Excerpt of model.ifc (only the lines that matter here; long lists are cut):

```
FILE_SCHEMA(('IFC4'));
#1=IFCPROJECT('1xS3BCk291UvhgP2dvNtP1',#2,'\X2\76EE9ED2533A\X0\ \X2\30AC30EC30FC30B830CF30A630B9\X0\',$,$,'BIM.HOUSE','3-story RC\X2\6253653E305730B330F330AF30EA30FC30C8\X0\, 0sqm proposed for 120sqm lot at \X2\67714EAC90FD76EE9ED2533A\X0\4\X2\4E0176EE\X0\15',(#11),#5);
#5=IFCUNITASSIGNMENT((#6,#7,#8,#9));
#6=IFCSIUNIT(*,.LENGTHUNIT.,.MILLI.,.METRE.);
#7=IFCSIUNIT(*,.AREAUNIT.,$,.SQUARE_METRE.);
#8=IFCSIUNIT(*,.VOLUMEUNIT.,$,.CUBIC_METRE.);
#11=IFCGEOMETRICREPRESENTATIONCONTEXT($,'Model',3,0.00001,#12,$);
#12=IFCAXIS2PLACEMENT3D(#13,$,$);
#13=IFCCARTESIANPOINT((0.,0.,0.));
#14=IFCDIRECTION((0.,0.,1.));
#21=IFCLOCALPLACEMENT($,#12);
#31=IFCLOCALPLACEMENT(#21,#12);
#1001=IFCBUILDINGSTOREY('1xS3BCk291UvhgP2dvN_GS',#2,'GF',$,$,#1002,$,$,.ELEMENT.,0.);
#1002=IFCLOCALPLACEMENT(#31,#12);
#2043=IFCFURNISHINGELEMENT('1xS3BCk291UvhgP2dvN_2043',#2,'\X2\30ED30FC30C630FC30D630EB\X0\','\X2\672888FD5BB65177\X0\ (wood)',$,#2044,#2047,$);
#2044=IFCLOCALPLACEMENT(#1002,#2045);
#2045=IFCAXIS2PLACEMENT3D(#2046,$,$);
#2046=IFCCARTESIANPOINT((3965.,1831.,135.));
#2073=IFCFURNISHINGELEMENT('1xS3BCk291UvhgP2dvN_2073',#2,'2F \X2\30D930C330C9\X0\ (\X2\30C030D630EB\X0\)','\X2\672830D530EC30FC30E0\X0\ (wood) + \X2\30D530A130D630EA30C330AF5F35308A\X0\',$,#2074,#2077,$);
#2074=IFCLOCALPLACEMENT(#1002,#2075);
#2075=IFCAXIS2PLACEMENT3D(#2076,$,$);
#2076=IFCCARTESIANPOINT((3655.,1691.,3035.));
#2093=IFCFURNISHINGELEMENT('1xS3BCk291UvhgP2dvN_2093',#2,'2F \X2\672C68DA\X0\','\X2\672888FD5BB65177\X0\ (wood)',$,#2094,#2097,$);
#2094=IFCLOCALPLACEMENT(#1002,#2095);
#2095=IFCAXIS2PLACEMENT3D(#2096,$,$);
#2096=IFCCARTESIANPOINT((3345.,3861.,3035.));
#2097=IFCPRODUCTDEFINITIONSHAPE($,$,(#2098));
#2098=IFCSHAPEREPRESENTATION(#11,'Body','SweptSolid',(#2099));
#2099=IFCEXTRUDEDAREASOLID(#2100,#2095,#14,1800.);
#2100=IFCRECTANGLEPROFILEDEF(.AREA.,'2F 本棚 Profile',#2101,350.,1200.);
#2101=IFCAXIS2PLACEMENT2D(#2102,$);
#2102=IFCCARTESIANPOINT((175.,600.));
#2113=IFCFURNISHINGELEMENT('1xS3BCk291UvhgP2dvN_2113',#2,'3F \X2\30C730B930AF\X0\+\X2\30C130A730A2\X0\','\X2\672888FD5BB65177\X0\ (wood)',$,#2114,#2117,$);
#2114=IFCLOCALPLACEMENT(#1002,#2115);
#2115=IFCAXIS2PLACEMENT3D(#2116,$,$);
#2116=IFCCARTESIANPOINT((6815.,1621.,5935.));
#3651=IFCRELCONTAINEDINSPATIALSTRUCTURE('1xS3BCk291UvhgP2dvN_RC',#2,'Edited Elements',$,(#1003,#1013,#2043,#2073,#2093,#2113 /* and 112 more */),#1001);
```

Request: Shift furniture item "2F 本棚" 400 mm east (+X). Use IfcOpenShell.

```python
import ifcopenshell
import ifcopenshell.api.geometry
import ifcopenshell.util.placement
import ifcopenshell.util.unit

model = ifcopenshell.open("model.ifc")
unit_scale = ifcopenshell.util.unit.calculate_unit_scale(model)

item = model.by_guid("1xS3BCk291UvhgP2dvN_2093")
matrix = ifcopenshell.util.placement.get_local_placement(item.ObjectPlacement)
matrix[0, 3] += 0.4 / unit_scale
ifcopenshell.api.geometry.edit_object_placement(model, product=item, matrix=matrix, is_si=False)

print(ifcopenshell.util.placement.get_local_placement(item.ObjectPlacement).round(3) + 0.0)

model.write("model-out.ifc")
```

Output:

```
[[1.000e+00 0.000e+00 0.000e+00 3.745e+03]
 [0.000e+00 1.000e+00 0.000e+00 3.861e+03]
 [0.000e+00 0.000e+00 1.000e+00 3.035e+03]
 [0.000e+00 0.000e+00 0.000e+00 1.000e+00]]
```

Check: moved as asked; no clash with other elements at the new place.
